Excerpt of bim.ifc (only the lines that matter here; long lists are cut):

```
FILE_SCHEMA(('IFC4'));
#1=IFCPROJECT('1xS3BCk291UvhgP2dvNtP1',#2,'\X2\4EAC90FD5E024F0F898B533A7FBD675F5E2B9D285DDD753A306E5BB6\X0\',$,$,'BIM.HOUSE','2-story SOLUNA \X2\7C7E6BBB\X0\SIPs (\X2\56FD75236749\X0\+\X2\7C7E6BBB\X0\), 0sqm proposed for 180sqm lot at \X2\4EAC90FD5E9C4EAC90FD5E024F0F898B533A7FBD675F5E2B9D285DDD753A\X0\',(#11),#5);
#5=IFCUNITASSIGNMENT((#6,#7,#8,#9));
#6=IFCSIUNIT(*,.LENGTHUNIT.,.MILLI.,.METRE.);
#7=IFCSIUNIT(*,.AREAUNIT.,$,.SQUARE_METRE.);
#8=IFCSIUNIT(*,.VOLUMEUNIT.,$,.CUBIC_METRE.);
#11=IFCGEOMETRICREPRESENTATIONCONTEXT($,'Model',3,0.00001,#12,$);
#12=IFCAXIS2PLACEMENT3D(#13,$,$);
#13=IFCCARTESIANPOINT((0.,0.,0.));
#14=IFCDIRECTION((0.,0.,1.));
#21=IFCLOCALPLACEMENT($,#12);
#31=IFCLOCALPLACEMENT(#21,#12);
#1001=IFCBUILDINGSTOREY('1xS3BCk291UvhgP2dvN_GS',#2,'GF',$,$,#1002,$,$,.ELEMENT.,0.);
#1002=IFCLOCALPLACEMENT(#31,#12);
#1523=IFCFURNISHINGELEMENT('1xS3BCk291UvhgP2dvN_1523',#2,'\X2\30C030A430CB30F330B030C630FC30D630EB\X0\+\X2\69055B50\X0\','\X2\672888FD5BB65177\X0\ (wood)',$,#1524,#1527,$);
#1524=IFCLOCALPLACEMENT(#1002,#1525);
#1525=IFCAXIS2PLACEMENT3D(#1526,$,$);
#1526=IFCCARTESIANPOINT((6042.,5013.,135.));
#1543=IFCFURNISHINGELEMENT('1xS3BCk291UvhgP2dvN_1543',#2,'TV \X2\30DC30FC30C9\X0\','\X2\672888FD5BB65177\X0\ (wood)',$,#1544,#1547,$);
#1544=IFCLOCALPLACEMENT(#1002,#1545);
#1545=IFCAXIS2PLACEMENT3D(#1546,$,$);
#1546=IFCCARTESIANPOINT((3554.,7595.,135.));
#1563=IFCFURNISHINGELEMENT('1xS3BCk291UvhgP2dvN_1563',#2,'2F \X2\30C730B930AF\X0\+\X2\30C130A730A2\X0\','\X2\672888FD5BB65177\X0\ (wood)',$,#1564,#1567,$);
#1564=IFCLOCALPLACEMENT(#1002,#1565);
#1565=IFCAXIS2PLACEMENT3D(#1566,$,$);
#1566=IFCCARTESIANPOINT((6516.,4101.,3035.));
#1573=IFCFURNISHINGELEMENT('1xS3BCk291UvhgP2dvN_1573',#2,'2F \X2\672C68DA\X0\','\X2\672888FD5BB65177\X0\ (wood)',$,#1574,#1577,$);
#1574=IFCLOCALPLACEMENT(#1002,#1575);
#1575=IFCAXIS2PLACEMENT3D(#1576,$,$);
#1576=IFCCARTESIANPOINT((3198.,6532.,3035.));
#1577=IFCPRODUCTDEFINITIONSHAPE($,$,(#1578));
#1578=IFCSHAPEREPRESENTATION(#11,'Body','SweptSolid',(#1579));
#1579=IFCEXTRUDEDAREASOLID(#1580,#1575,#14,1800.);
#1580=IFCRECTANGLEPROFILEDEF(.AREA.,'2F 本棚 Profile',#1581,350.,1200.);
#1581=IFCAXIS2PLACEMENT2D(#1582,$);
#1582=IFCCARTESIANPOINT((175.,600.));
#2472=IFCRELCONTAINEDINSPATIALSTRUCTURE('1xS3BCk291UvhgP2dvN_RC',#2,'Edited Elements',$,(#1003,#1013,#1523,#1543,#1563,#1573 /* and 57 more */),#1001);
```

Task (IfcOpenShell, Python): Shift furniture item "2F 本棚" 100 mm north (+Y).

```python
import ifcopenshell
import ifcopenshell.api.geometry
import ifcopenshell.util.placement
import ifcopenshell.util.unit

model = ifcopenshell.open("bim.ifc")
unit_scale = ifcopenshell.util.unit.calculate_unit_scale(model)

item = model.by_guid("1xS3BCk291UvhgP2dvN_1573")
matrix = ifcopenshell.util.placement.get_local_placement(item.ObjectPlacement)
matrix[1, 3] += 0.1 / unit_scale
ifcopenshell.api.geometry.edit_object_placement(model, product=item, matrix=matrix, is_si=False)

print(ifcopenshell.util.placement.get_local_placement(item.ObjectPlacement).round(3) + 0.0)

model.write("bim-out.ifc")
```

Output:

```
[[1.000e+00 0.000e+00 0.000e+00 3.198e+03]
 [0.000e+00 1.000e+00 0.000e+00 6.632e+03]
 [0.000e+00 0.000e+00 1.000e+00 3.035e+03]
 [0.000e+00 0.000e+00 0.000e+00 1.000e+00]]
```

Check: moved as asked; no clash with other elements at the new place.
